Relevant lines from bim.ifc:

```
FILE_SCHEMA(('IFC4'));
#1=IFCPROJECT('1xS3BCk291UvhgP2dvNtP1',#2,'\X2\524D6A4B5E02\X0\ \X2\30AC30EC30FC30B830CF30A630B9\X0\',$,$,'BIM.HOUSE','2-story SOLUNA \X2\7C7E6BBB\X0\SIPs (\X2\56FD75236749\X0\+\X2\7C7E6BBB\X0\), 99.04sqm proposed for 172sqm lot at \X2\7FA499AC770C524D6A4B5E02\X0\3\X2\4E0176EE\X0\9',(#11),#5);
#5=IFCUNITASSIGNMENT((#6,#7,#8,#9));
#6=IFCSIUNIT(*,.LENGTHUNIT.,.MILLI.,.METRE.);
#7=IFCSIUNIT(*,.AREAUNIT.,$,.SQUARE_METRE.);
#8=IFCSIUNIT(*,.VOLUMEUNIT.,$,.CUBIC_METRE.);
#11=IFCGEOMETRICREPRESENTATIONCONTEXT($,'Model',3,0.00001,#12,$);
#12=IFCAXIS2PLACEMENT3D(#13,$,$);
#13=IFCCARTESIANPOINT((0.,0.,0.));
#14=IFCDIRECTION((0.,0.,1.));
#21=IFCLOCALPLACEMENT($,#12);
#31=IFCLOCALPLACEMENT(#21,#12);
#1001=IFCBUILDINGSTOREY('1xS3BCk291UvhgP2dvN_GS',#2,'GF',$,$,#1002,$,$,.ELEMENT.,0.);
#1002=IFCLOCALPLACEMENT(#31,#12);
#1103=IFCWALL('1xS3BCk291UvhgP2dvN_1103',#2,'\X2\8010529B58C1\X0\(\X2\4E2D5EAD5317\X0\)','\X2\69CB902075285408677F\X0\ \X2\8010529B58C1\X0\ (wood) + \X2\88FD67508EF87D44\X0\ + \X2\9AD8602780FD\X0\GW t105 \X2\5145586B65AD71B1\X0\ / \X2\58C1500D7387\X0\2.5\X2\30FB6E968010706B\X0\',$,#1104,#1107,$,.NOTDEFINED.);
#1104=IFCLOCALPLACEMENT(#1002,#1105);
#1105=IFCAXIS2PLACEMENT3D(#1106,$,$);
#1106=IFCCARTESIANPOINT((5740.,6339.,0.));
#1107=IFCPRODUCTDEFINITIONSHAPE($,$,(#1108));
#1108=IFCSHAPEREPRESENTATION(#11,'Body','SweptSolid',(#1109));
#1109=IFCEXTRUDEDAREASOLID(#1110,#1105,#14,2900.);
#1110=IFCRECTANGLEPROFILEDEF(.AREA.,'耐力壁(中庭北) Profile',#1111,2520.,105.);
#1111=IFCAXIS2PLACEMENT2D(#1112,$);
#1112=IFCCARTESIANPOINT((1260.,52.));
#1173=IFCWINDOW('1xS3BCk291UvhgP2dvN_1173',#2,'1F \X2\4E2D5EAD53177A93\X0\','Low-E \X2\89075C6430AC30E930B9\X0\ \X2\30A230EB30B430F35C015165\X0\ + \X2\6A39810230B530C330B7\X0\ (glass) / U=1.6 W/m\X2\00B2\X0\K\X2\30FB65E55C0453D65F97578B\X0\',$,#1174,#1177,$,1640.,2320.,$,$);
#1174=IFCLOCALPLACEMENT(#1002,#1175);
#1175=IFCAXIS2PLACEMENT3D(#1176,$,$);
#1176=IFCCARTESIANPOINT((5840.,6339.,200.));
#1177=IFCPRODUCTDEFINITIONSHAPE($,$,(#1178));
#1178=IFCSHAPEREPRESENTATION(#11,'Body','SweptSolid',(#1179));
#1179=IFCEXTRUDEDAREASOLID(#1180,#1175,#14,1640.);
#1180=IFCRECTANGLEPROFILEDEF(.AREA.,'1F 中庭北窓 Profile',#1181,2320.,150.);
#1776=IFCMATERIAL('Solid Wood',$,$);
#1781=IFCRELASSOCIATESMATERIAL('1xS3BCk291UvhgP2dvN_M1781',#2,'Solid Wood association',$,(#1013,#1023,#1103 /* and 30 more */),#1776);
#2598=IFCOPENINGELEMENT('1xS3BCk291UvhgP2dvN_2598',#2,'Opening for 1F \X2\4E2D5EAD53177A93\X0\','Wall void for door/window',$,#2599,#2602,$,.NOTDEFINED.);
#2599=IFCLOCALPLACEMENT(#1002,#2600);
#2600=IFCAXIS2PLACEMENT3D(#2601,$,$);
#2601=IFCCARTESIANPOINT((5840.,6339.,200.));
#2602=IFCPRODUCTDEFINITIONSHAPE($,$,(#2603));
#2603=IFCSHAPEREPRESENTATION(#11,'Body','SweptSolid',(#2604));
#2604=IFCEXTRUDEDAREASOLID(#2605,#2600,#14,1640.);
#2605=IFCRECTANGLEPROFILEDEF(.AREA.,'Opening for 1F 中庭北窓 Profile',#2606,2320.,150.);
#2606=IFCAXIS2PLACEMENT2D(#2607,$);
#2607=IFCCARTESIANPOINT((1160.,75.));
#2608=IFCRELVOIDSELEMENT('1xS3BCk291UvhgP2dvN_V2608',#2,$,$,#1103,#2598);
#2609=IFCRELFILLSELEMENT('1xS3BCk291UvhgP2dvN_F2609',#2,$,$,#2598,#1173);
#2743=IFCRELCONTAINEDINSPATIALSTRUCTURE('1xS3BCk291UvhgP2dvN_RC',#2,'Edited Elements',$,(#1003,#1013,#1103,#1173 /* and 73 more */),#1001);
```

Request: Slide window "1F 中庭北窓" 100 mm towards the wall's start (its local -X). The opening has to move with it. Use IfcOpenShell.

```python
import ifcopenshell
import ifcopenshell.api.geometry
import ifcopenshell.util.placement
import ifcopenshell.util.unit

model = ifcopenshell.open("bim.ifc")
unit_scale = ifcopenshell.util.unit.calculate_unit_scale(model)

window = model.by_guid("1xS3BCk291UvhgP2dvN_1173")
opening = window.FillsVoids[0].RelatingOpeningElement
wall = opening.VoidsElements[0].RelatingBuildingElement

wall_matrix = ifcopenshell.util.placement.get_local_placement(wall.ObjectPlacement)
shift = wall_matrix[:3, 0] * -0.1 / unit_scale
before = ifcopenshell.util.placement.get_local_placement(window.ObjectPlacement)[:3, 3].copy()

# The window is not placed relative to its opening, so move both.
for product in (opening, window):
    matrix = ifcopenshell.util.placement.get_local_placement(product.ObjectPlacement)
    matrix[:3, 3] += shift
    ifcopenshell.api.geometry.edit_object_placement(model, product=product, matrix=matrix, is_si=False)

after = ifcopenshell.util.placement.get_local_placement(window.ObjectPlacement)[:3, 3]
print("window moved by", (after - before).round(3) + 0.0)

model.write("bim-out.ifc")
```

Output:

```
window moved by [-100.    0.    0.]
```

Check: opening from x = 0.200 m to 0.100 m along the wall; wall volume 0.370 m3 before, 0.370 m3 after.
